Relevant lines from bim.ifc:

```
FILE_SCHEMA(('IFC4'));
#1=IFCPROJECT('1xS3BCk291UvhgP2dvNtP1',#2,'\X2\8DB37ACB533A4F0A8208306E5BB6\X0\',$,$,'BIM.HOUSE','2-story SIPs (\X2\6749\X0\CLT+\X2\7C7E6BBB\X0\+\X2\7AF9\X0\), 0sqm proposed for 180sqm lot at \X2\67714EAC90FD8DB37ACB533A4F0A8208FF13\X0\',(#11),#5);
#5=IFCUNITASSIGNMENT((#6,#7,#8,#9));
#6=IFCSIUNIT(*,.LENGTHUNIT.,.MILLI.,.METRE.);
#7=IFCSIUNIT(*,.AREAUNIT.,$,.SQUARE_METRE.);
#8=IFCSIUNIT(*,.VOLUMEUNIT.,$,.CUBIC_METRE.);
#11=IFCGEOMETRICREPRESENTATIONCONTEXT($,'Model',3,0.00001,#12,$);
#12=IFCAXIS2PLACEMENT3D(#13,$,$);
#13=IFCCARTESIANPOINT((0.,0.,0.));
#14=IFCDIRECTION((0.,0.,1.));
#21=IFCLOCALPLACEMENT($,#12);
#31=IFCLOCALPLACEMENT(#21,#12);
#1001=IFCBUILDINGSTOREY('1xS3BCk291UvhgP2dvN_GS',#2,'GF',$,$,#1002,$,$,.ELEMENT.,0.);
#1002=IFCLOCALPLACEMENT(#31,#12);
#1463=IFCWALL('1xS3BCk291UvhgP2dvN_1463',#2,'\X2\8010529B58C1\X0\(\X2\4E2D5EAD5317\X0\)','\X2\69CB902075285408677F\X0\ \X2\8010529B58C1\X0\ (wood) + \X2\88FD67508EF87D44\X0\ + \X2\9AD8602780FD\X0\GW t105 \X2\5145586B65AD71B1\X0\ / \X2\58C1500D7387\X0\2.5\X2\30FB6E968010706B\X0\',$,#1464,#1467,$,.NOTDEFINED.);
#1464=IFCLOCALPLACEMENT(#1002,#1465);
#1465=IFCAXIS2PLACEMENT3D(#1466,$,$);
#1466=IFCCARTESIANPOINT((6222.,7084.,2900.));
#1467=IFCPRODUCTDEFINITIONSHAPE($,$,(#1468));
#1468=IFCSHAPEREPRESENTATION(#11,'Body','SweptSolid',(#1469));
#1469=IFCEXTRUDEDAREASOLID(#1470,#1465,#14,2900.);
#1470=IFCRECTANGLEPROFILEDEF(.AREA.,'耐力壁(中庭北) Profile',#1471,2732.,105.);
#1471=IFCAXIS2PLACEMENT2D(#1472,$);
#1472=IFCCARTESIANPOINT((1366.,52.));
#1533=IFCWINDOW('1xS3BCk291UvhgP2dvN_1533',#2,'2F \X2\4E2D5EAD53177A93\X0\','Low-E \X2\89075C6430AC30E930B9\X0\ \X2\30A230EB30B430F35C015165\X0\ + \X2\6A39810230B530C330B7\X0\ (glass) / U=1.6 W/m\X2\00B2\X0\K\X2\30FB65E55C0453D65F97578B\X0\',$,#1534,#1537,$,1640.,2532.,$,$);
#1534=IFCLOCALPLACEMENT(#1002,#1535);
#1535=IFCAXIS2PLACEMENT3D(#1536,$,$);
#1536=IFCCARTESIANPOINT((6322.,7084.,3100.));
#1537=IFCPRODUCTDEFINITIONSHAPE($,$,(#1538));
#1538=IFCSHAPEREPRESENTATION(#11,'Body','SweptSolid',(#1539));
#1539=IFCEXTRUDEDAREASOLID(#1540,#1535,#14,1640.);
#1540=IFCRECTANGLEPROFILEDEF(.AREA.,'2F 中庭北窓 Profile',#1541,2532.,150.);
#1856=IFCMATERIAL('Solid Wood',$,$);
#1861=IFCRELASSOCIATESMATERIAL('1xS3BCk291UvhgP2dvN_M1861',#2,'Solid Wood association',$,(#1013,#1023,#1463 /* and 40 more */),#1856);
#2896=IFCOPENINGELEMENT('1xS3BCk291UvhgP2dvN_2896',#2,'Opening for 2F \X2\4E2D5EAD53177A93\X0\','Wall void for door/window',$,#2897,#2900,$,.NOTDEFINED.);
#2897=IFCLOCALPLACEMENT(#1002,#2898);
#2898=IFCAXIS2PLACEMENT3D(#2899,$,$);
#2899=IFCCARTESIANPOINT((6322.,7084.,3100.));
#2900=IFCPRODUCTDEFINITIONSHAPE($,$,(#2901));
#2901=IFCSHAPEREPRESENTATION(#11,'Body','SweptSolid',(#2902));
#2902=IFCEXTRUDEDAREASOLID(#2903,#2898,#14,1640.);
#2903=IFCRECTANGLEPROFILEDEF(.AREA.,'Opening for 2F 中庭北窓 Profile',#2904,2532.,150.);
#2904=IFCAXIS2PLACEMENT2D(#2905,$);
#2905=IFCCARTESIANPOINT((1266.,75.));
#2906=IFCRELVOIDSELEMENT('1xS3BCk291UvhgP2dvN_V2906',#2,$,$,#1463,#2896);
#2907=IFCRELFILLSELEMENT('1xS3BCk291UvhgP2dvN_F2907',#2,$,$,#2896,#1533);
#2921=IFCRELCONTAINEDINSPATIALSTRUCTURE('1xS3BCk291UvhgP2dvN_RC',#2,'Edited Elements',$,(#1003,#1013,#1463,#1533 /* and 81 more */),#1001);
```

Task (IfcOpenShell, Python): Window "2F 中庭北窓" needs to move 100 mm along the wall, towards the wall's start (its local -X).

```python
import ifcopenshell
import ifcopenshell.api.geometry
import ifcopenshell.util.placement
import ifcopenshell.util.unit

model = ifcopenshell.open("bim.ifc")
unit_scale = ifcopenshell.util.unit.calculate_unit_scale(model)

window = model.by_guid("1xS3BCk291UvhgP2dvN_1533")
opening = window.FillsVoids[0].RelatingOpeningElement
wall = opening.VoidsElements[0].RelatingBuildingElement

wall_matrix = ifcopenshell.util.placement.get_local_placement(wall.ObjectPlacement)
shift = wall_matrix[:3, 0] * -0.1 / unit_scale
before = ifcopenshell.util.placement.get_local_placement(window.ObjectPlacement)[:3, 3].copy()

# The window is not placed relative to its opening, so move both.
for product in (opening, window):
    matrix = ifcopenshell.util.placement.get_local_placement(product.ObjectPlacement)
    matrix[:3, 3] += shift
    ifcopenshell.api.geometry.edit_object_placement(model, product=product, matrix=matrix, is_si=False)

after = ifcopenshell.util.placement.get_local_placement(window.ObjectPlacement)[:3, 3]
print("window moved by", (after - before).round(3) + 0.0)

model.write("bim_edited.ifc")
```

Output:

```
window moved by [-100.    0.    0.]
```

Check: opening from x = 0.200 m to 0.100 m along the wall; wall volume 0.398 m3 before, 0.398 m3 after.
